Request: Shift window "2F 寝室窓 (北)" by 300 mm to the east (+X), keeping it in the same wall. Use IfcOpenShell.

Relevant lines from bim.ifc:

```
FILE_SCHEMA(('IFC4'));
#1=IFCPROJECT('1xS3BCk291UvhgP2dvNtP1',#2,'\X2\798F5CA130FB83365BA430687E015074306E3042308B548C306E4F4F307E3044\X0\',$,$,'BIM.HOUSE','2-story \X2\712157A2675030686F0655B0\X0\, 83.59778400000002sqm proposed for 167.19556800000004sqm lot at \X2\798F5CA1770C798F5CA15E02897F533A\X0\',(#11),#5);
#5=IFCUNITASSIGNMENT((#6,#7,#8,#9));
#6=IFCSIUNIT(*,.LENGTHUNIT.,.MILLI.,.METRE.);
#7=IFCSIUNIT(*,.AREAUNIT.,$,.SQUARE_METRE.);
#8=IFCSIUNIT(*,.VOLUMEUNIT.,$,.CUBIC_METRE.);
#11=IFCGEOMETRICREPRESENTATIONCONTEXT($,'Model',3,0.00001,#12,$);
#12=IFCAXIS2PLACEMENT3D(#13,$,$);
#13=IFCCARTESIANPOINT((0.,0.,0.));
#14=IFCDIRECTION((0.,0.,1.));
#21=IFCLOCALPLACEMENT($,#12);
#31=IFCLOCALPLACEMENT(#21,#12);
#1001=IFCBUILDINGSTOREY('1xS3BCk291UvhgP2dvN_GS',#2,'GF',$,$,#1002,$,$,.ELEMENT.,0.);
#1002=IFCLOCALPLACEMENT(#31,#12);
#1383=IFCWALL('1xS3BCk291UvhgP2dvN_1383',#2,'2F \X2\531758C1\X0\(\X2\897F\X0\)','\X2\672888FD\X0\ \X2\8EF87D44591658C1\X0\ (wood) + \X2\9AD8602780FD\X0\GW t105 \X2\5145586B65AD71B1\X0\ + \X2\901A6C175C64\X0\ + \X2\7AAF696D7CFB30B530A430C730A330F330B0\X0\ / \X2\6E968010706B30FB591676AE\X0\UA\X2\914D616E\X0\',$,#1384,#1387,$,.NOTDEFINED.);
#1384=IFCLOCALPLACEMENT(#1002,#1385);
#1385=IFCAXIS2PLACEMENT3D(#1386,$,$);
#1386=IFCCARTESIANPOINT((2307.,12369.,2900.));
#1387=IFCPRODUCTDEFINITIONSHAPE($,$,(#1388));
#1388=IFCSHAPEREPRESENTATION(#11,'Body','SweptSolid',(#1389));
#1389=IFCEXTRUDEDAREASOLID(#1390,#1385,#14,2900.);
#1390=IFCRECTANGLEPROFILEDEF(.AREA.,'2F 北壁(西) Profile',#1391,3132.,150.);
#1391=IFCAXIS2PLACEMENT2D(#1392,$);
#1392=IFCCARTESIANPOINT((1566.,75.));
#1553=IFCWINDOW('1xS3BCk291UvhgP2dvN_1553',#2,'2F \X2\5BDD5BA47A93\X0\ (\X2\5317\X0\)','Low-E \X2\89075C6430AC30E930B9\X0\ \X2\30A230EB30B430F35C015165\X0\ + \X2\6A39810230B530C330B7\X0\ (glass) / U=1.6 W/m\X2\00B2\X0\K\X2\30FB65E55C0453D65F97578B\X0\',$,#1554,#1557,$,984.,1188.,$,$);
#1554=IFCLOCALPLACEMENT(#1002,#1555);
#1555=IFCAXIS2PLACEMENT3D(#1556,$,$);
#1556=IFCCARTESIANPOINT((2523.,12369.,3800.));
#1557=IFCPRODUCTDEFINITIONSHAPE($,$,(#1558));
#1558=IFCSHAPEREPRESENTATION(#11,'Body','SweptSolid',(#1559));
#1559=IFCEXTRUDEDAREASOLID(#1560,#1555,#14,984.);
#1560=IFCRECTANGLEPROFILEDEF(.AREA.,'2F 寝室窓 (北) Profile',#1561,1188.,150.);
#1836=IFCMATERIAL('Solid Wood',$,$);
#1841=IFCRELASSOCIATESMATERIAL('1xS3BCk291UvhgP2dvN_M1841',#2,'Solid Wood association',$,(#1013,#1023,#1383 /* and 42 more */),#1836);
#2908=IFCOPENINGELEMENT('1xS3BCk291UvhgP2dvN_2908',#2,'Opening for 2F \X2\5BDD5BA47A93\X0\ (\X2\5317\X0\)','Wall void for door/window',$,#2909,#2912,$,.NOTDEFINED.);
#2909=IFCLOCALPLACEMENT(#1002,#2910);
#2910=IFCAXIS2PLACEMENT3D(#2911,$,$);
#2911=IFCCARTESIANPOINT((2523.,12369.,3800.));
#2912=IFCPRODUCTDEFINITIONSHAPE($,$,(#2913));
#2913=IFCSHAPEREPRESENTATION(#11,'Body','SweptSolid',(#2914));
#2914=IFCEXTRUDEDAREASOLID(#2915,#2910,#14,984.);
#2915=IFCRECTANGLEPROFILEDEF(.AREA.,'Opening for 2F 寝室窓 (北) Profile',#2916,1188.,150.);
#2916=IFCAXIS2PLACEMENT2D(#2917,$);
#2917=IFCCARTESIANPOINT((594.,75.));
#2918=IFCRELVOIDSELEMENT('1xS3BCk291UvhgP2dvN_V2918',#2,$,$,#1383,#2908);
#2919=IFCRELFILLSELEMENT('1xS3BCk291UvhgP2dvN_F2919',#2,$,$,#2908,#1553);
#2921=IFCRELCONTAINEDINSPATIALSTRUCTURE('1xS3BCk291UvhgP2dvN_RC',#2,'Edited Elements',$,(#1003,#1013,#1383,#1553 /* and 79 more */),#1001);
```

```python
import ifcopenshell
import ifcopenshell.api.geometry
import ifcopenshell.util.placement
import ifcopenshell.util.unit

model = ifcopenshell.open("bim.ifc")
unit_scale = ifcopenshell.util.unit.calculate_unit_scale(model)

window = model.by_id(1553)
opening = window.FillsVoids[0].RelatingOpeningElement
wall = opening.VoidsElements[0].RelatingBuildingElement

wall_matrix = ifcopenshell.util.placement.get_local_placement(wall.ObjectPlacement)
shift = wall_matrix[:3, 0] * 0.3 / unit_scale
before = ifcopenshell.util.placement.get_local_placement(window.ObjectPlacement)[:3, 3].copy()

# The window is not placed relative to its opening, so move both.
for product in (opening, window):
    matrix = ifcopenshell.util.placement.get_local_placement(product.ObjectPlacement)
    matrix[:3, 3] += shift
    ifcopenshell.api.geometry.edit_object_placement(model, product=product, matrix=matrix, is_si=False)

after = ifcopenshell.util.placement.get_local_placement(window.ObjectPlacement)[:3, 3]
print("window moved by", (after - before).round(3) + 0.0)

model.write("bim_v2.ifc")
```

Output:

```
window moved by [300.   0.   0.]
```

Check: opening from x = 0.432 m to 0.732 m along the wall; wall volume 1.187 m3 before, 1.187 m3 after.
